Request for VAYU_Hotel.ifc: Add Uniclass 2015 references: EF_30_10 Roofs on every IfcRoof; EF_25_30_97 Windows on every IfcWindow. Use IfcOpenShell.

First a look at what the model holds.

```python
import ifcopenshell

model = ifcopenshell.open("VAYU_Hotel.ifc")
print(model.schema)
print("classifications:", [c.Name for c in model.by_type("IfcClassification")])
for ifc_class in ("IfcDoor", "IfcRoof", "IfcStair", "IfcWall", "IfcWindow"):
    print(ifc_class, len(model.by_type(ifc_class)))
```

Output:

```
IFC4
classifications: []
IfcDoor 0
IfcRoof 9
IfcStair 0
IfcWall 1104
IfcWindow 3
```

```python
import ifcopenshell
import ifcopenshell.api.classification

model = ifcopenshell.open("VAYU_Hotel.ifc")

system = ifcopenshell.api.classification.add_classification(model, classification="Uniclass 2015")

codes = {
    "IfcRoof": ("EF_30_10", "Roofs"),
    "IfcWindow": ("EF_25_30_97", "Windows"),
}
for ifc_class, (code, name) in codes.items():
    products = model.by_type(ifc_class)
    ifcopenshell.api.classification.add_reference(
        model, products=products, classification=system, identification=code, name=name
    )
    print(code, len(products))

model.write("VAYU_Hotel_v2.ifc")
```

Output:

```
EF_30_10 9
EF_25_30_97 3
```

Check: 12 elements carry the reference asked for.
